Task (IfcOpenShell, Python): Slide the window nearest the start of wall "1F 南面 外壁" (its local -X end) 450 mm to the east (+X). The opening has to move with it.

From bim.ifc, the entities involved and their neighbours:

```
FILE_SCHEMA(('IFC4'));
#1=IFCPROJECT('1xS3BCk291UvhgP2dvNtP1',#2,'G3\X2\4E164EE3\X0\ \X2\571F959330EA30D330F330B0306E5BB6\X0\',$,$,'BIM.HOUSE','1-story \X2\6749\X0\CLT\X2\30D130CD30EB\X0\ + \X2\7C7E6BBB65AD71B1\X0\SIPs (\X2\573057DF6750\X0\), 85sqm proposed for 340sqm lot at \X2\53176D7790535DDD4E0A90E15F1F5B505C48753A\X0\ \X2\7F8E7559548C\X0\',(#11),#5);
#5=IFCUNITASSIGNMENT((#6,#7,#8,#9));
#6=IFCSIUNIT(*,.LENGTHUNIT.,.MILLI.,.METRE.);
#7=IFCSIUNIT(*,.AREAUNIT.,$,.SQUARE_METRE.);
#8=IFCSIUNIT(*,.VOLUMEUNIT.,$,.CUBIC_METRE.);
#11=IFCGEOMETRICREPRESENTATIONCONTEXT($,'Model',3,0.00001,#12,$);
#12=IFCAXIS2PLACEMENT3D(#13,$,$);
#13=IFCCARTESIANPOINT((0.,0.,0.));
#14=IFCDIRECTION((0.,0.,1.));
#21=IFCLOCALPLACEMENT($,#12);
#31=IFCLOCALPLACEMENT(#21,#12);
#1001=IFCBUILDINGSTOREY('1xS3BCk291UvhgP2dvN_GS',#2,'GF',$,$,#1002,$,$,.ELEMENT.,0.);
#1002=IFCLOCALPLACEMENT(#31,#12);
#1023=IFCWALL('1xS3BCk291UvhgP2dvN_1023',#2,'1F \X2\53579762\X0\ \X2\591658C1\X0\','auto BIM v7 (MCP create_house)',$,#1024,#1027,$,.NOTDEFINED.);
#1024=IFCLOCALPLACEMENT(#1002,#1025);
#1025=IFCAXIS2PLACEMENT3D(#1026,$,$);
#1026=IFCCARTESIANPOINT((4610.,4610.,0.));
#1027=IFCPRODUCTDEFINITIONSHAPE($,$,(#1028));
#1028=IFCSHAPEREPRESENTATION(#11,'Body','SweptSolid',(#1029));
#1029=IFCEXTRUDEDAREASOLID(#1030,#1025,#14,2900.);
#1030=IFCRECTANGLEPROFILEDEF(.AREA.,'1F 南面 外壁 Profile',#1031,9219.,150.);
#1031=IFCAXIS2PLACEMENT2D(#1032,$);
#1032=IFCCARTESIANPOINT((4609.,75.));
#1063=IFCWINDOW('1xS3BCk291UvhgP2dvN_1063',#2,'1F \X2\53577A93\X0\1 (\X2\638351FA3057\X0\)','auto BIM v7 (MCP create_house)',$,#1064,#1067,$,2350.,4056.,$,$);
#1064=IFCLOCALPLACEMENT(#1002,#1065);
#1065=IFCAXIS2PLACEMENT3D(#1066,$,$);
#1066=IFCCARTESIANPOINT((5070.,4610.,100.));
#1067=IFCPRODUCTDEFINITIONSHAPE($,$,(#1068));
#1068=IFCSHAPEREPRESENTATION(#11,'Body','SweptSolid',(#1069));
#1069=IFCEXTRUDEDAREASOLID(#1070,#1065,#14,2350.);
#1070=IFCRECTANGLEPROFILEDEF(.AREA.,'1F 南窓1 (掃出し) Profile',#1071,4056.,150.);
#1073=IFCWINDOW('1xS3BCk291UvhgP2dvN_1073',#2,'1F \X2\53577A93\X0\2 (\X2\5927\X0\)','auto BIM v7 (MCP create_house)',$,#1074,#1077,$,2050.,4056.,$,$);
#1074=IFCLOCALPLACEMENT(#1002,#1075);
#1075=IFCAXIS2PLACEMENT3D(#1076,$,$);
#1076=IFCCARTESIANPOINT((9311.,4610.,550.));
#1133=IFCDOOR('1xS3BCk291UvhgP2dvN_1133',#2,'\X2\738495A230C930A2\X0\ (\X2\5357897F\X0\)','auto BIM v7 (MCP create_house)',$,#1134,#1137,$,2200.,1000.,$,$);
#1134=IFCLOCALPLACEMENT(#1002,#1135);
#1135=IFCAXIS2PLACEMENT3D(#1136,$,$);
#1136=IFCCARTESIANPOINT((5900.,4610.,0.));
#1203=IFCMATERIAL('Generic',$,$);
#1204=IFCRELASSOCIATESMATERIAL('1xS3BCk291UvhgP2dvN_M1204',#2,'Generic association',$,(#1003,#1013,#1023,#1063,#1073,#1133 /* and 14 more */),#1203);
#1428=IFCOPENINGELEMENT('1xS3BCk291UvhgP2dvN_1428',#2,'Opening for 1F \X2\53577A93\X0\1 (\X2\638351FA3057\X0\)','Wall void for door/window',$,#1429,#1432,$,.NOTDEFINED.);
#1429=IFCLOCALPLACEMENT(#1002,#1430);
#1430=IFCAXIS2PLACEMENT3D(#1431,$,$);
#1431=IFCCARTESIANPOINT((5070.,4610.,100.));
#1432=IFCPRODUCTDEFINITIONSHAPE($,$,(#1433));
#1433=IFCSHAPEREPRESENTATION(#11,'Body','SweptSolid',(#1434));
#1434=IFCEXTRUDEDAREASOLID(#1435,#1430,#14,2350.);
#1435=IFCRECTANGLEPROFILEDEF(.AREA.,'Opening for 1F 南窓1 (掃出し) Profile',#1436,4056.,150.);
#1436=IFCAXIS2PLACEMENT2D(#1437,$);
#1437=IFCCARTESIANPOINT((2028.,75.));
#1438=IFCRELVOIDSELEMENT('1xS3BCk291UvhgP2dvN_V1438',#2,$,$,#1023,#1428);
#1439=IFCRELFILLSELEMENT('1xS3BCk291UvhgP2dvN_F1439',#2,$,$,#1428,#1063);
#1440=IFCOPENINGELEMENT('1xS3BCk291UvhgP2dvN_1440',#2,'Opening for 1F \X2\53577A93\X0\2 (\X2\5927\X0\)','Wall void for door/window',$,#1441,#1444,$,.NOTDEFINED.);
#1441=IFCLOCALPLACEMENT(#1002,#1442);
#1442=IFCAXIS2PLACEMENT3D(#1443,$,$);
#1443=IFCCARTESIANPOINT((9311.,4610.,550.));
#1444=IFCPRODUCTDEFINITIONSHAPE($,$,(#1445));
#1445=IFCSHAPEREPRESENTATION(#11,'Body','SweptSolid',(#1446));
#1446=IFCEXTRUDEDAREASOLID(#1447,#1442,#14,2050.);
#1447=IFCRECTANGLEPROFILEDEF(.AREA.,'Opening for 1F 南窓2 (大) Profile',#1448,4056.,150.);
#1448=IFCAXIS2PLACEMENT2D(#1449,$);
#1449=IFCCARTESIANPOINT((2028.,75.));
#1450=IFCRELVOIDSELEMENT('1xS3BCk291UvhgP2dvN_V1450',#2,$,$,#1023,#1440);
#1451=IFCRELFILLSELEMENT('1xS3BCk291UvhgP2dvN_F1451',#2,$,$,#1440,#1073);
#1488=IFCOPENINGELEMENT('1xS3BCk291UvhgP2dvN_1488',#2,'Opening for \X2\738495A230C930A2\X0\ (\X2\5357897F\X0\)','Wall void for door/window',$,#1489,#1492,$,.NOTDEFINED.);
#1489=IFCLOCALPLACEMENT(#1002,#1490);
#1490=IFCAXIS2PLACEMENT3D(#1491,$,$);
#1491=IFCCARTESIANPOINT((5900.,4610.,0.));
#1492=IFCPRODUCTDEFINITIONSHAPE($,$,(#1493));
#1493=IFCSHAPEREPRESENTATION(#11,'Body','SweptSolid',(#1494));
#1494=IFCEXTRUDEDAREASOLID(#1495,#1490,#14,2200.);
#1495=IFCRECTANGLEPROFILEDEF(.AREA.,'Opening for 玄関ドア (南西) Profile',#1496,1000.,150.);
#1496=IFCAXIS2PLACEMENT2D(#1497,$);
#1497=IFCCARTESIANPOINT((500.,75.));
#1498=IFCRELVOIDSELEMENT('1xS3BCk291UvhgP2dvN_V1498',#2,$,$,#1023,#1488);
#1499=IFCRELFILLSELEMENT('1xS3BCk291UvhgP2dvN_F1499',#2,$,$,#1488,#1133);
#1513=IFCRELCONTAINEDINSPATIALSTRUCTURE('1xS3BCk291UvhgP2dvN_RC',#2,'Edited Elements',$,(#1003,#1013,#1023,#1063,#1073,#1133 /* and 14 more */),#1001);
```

```python
import ifcopenshell
import ifcopenshell.api.geometry
import ifcopenshell.util.placement
import ifcopenshell.util.unit

model = ifcopenshell.open("bim.ifc")
unit_scale = ifcopenshell.util.unit.calculate_unit_scale(model)

window = model.by_guid("1xS3BCk291UvhgP2dvN_1063")
opening = window.FillsVoids[0].RelatingOpeningElement
wall = opening.VoidsElements[0].RelatingBuildingElement

wall_matrix = ifcopenshell.util.placement.get_local_placement(wall.ObjectPlacement)
shift = wall_matrix[:3, 0] * 0.45 / unit_scale
before = ifcopenshell.util.placement.get_local_placement(window.ObjectPlacement)[:3, 3].copy()

# The window is not placed relative to its opening, so move both.
for product in (opening, window):
    matrix = ifcopenshell.util.placement.get_local_placement(product.ObjectPlacement)
    matrix[:3, 3] += shift
    ifcopenshell.api.geometry.edit_object_placement(model, product=product, matrix=matrix, is_si=False)

after = ifcopenshell.util.placement.get_local_placement(window.ObjectPlacement)[:3, 3]
print("window moved by", (after - before).round(3) + 0.0)

model.write("bim_rev.ifc")
```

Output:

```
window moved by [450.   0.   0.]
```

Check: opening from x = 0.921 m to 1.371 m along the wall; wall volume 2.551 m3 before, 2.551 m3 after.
